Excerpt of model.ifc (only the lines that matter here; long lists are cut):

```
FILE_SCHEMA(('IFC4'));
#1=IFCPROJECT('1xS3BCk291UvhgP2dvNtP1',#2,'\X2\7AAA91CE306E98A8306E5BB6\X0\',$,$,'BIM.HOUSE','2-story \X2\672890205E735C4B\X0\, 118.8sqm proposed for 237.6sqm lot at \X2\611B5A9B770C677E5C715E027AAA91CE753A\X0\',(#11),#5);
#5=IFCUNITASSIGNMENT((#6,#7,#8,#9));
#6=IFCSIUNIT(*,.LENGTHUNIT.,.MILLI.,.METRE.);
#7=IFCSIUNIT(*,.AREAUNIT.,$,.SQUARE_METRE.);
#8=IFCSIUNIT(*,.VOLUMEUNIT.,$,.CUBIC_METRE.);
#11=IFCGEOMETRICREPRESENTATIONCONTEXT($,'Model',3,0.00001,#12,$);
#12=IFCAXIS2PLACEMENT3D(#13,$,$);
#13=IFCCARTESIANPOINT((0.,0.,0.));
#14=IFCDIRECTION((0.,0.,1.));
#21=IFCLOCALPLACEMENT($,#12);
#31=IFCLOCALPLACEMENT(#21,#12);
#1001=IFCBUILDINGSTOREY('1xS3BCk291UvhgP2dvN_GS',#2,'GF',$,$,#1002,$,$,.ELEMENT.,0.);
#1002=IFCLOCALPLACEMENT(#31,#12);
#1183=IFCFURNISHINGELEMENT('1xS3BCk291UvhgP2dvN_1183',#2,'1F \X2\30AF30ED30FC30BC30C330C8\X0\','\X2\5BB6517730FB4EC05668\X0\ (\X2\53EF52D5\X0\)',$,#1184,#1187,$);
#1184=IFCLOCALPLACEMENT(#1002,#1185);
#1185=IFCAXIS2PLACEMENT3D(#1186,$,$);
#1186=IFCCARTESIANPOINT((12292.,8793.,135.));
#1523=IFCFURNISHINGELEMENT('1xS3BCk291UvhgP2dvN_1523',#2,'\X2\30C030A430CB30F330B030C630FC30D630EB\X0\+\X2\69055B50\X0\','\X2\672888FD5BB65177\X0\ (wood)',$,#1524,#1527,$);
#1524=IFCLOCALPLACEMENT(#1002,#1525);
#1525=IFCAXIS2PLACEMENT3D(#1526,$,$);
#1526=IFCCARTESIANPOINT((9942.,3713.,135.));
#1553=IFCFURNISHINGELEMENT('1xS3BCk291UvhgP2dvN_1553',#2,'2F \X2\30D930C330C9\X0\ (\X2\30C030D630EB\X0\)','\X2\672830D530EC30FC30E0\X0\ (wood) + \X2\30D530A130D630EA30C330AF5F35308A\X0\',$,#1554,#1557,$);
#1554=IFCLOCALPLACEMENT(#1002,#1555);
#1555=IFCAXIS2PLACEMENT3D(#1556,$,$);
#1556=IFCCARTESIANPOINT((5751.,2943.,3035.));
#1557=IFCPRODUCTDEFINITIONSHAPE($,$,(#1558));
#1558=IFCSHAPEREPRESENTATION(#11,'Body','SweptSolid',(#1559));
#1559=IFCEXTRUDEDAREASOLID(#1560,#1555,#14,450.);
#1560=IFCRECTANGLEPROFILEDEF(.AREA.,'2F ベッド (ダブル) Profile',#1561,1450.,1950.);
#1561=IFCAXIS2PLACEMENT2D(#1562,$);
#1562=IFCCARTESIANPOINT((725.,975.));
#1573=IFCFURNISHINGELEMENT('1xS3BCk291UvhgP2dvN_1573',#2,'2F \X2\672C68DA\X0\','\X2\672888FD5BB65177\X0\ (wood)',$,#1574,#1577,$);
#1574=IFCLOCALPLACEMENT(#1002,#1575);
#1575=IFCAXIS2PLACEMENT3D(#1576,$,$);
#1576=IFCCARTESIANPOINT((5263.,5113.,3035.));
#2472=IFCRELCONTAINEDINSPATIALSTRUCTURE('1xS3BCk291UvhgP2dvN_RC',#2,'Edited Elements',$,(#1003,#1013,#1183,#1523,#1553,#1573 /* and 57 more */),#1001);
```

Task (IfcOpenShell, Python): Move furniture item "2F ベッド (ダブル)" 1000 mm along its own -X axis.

```python
import ifcopenshell
import ifcopenshell.api.geometry
import ifcopenshell.util.placement
import ifcopenshell.util.unit

model = ifcopenshell.open("model.ifc")
unit_scale = ifcopenshell.util.unit.calculate_unit_scale(model)

item = model.by_id(1553)
matrix = ifcopenshell.util.placement.get_local_placement(item.ObjectPlacement)
matrix[:3, 3] -= matrix[:3, 0] * 1 / unit_scale
ifcopenshell.api.geometry.edit_object_placement(model, product=item, matrix=matrix, is_si=False)

print(ifcopenshell.util.placement.get_local_placement(item.ObjectPlacement).round(3) + 0.0)

model.write("model-out.ifc")
```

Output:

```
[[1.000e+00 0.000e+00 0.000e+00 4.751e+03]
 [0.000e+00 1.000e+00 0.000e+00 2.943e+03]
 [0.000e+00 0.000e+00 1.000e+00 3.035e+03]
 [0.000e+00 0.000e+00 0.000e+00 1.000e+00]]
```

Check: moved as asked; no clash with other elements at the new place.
